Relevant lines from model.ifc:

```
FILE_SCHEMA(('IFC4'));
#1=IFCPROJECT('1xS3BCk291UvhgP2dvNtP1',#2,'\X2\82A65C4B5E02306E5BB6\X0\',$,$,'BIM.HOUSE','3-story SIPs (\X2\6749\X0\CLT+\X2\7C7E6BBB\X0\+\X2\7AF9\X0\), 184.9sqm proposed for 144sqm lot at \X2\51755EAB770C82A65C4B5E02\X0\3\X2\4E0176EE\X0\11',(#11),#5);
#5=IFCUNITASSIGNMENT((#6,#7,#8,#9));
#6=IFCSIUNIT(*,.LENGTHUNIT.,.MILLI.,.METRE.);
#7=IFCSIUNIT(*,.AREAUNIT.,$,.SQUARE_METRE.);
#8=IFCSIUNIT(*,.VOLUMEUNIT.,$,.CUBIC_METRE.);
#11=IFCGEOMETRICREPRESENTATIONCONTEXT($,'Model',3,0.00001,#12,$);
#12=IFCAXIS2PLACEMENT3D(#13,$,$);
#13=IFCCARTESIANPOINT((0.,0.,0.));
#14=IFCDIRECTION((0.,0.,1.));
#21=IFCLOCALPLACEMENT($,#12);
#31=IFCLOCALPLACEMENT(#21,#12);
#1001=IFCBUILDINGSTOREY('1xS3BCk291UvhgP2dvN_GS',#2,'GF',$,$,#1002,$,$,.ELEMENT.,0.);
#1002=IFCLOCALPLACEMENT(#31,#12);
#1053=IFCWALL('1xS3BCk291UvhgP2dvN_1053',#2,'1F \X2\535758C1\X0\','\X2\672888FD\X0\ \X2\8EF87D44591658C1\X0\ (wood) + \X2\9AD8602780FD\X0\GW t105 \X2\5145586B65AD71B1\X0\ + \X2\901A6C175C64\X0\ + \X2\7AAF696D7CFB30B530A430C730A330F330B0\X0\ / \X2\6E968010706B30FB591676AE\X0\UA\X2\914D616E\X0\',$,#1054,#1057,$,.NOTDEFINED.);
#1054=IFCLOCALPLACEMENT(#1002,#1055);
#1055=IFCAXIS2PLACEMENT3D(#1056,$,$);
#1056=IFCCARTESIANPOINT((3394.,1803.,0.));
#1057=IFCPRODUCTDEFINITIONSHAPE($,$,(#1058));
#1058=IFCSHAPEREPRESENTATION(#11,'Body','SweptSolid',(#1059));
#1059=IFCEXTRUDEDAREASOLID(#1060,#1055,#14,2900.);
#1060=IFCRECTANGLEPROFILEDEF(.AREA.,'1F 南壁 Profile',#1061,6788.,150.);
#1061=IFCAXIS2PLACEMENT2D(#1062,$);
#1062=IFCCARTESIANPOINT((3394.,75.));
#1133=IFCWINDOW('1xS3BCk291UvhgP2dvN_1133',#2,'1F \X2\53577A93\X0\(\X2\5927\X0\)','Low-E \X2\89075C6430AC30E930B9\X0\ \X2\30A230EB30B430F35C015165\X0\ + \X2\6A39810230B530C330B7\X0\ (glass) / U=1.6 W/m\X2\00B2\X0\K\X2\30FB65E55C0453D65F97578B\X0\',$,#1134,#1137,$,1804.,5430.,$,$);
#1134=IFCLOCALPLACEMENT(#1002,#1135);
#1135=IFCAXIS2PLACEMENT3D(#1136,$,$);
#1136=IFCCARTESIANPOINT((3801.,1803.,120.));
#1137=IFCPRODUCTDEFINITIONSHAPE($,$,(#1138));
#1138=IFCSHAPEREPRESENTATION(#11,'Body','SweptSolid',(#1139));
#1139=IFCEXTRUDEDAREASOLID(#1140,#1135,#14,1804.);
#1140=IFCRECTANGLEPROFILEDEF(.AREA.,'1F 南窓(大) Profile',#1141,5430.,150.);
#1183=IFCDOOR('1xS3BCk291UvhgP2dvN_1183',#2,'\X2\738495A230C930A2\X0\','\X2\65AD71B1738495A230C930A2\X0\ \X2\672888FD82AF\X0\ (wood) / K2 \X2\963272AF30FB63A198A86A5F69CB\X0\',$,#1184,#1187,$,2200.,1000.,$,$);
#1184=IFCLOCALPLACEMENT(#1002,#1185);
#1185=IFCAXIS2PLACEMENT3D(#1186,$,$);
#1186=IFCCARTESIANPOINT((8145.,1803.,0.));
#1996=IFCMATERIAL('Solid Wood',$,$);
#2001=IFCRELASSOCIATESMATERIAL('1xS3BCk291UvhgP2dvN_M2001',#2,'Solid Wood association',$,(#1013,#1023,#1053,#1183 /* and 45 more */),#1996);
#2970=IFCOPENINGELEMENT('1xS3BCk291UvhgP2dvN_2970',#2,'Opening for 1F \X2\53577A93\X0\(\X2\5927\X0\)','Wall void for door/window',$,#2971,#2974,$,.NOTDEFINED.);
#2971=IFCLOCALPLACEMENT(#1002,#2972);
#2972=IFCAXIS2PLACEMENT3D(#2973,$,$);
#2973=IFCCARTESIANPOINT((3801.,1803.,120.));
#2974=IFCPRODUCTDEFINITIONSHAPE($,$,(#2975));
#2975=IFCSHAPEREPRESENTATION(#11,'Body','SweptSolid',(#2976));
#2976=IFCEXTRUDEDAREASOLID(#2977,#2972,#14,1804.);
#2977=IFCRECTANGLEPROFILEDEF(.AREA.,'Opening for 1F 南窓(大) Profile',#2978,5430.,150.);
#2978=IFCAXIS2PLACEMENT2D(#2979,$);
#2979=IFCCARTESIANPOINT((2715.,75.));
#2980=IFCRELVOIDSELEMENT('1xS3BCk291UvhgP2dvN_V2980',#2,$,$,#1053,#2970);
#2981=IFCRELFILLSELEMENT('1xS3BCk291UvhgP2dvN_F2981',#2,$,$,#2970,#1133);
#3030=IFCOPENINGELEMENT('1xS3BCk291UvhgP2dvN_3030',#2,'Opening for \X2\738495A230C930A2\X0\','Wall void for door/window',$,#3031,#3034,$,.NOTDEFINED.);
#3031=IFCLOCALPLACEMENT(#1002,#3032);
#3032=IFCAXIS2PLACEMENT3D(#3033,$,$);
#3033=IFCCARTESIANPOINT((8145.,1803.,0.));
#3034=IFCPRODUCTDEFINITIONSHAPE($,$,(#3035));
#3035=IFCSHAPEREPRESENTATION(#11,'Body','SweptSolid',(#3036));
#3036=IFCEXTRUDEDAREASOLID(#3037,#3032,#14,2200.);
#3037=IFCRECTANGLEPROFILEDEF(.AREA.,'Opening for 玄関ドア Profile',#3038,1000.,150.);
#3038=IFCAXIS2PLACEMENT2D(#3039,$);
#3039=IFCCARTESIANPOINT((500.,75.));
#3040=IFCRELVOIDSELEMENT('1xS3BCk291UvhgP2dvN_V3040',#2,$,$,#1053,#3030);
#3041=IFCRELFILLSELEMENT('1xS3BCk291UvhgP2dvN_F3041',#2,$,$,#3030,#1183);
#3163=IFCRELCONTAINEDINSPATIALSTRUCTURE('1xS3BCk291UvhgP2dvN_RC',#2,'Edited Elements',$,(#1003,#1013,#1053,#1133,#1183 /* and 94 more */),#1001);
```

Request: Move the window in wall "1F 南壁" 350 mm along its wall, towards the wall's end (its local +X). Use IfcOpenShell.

```python
import ifcopenshell
import ifcopenshell.api.geometry
import ifcopenshell.util.placement

model = ifcopenshell.open("model.ifc")

window = model.by_id(1133)
opening = window.FillsVoids[0].RelatingOpeningElement
wall = opening.VoidsElements[0].RelatingBuildingElement

wall_matrix = ifcopenshell.util.placement.get_local_placement(wall.ObjectPlacement)
shift = wall_matrix[:3, 0] * 350.0
before = ifcopenshell.util.placement.get_local_placement(window.ObjectPlacement)[:3, 3].copy()

# The window is not placed relative to its opening, so move both.
for product in (opening, window):
    matrix = ifcopenshell.util.placement.get_local_placement(product.ObjectPlacement)
    matrix[:3, 3] += shift
    ifcopenshell.api.geometry.edit_object_placement(model, product=product, matrix=matrix, is_si=False)

after = ifcopenshell.util.placement.get_local_placement(window.ObjectPlacement)[:3, 3]
print("window moved by", (after - before).round(3) + 0.0)

model.write("model_rev.ifc")
```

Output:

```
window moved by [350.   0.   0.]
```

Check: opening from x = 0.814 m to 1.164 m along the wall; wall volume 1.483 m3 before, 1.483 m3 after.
